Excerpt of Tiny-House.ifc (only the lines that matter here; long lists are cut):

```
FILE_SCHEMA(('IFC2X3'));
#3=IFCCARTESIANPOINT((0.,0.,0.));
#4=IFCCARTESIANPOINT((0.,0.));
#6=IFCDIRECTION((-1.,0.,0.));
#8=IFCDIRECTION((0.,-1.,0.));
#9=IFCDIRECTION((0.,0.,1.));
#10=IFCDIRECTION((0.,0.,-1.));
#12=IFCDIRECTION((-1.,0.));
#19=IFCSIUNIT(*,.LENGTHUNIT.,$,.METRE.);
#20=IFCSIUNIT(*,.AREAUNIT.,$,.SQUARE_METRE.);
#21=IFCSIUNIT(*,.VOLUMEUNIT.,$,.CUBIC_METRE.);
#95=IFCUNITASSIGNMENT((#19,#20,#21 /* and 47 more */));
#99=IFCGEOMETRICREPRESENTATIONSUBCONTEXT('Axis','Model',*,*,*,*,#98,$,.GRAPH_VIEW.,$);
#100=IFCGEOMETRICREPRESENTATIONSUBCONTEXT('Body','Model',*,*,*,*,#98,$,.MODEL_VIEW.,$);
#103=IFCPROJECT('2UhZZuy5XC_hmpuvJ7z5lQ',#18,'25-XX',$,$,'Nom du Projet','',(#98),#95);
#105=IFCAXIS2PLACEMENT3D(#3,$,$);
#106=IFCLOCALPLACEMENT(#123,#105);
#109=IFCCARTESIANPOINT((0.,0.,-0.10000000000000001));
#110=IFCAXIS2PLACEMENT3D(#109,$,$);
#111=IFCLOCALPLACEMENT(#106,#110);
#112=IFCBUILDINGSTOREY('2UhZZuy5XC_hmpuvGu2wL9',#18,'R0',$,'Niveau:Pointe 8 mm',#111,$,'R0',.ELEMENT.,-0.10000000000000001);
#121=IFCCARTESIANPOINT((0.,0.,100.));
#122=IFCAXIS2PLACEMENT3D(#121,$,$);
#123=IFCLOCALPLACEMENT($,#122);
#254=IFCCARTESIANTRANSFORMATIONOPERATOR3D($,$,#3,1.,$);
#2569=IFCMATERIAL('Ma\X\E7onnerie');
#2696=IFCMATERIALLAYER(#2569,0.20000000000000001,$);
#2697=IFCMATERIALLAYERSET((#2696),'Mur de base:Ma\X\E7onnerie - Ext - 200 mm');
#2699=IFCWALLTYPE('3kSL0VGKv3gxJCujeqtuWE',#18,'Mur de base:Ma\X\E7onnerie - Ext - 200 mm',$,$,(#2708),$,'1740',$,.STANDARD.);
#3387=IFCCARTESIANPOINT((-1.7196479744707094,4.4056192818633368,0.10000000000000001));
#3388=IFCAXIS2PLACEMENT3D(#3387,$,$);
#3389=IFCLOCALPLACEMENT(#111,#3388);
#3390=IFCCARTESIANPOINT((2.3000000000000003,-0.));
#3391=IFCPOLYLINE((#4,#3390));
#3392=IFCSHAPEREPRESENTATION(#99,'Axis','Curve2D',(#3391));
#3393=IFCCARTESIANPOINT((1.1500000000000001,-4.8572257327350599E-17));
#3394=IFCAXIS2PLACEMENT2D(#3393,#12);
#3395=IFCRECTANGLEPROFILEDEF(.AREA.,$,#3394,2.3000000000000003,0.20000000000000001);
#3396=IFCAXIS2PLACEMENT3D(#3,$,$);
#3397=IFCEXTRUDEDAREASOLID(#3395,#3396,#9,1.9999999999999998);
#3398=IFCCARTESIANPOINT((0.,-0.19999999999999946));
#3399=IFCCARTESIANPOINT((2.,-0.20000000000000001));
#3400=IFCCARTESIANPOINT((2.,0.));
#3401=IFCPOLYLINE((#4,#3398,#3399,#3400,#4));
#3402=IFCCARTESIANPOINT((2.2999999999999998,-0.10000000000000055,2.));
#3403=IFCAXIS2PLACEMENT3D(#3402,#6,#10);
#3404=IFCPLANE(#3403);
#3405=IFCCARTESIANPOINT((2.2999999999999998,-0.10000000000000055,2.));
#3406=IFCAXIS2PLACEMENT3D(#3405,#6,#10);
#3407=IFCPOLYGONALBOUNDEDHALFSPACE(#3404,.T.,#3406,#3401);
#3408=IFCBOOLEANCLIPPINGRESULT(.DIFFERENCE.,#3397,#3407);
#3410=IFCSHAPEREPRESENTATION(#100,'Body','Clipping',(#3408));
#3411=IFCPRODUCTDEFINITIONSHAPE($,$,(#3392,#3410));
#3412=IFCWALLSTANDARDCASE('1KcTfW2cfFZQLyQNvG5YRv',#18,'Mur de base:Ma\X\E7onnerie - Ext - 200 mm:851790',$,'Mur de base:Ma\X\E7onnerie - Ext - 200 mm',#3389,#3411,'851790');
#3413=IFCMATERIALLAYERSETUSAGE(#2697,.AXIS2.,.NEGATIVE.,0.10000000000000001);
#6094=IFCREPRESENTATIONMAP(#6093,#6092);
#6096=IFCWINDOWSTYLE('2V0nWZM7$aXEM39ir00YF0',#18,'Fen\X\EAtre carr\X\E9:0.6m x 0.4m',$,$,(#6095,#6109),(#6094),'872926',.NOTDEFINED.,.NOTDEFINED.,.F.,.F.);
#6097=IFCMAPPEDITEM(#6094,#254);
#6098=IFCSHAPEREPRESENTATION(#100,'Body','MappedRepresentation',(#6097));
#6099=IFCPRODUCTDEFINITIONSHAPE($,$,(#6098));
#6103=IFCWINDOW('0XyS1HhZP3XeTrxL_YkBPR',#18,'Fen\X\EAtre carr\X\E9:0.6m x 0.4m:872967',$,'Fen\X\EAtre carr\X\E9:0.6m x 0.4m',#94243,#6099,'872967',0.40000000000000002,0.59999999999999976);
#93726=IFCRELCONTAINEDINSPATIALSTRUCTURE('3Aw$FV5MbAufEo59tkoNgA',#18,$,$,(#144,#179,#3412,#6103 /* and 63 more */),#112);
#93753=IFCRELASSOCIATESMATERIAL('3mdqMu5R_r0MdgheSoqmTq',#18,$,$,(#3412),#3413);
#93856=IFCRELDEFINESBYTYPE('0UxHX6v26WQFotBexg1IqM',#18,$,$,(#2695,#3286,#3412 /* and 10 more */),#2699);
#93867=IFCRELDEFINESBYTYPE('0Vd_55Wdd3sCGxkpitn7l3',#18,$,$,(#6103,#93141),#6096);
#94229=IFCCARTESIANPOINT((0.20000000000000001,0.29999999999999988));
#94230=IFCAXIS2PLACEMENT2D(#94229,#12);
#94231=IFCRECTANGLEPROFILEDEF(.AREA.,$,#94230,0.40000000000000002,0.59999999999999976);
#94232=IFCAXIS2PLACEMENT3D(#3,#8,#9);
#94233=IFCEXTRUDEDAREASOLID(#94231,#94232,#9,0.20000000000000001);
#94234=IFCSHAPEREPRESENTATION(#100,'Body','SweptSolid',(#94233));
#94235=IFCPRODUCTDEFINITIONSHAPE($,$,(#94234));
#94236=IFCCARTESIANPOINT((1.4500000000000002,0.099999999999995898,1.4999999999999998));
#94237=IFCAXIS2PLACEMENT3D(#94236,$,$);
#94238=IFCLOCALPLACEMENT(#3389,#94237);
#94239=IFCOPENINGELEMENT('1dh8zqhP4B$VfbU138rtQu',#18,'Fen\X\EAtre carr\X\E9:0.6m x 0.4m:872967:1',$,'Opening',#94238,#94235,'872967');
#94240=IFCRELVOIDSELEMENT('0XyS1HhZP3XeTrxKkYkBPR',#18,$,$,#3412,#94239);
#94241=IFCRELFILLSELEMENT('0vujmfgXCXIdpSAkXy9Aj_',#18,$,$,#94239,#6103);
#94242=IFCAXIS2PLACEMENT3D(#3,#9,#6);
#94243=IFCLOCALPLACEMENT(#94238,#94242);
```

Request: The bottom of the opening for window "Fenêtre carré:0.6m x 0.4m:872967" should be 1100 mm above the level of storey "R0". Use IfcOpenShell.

```python
import numpy as np
import ifcopenshell
import ifcopenshell.api.geometry
import ifcopenshell.geom
import ifcopenshell.util.element
import ifcopenshell.util.placement
import ifcopenshell.util.shape
import ifcopenshell.util.unit

model = ifcopenshell.open("Tiny-House.ifc")
unit_scale = ifcopenshell.util.unit.calculate_unit_scale(model)

window = model.by_guid("0XyS1HhZP3XeTrxL_YkBPR")
opening = window.FillsVoids[0].RelatingOpeningElement
storey = ifcopenshell.util.element.get_container(window, ifc_class="IfcBuildingStorey")
level = ifcopenshell.util.placement.get_local_placement(storey.ObjectPlacement)[2, 3]

# The opening's origin need not be at the sill, so measure its lowest point.
shape = ifcopenshell.geom.create_shape(ifcopenshell.geom.settings(), opening)
bottom = ifcopenshell.util.shape.get_shape_bottom_elevation(shape, shape.geometry) / unit_scale
dz = level + 1.1 / unit_scale - bottom

shift = np.array([0.0, 0.0, dz])
# The window is placed relative to its opening, so it follows when the opening moves.
matrix = ifcopenshell.util.placement.get_local_placement(opening.ObjectPlacement)
matrix[:3, 3] += shift
ifcopenshell.api.geometry.edit_object_placement(
    model, product=opening, matrix=matrix, is_si=False, should_transform_children=True
)

print(f"moved by {dz * unit_scale:+.3f} m")

model.write("Tiny-House_v2.ifc")
```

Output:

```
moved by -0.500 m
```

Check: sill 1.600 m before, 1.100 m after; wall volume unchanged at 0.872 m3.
